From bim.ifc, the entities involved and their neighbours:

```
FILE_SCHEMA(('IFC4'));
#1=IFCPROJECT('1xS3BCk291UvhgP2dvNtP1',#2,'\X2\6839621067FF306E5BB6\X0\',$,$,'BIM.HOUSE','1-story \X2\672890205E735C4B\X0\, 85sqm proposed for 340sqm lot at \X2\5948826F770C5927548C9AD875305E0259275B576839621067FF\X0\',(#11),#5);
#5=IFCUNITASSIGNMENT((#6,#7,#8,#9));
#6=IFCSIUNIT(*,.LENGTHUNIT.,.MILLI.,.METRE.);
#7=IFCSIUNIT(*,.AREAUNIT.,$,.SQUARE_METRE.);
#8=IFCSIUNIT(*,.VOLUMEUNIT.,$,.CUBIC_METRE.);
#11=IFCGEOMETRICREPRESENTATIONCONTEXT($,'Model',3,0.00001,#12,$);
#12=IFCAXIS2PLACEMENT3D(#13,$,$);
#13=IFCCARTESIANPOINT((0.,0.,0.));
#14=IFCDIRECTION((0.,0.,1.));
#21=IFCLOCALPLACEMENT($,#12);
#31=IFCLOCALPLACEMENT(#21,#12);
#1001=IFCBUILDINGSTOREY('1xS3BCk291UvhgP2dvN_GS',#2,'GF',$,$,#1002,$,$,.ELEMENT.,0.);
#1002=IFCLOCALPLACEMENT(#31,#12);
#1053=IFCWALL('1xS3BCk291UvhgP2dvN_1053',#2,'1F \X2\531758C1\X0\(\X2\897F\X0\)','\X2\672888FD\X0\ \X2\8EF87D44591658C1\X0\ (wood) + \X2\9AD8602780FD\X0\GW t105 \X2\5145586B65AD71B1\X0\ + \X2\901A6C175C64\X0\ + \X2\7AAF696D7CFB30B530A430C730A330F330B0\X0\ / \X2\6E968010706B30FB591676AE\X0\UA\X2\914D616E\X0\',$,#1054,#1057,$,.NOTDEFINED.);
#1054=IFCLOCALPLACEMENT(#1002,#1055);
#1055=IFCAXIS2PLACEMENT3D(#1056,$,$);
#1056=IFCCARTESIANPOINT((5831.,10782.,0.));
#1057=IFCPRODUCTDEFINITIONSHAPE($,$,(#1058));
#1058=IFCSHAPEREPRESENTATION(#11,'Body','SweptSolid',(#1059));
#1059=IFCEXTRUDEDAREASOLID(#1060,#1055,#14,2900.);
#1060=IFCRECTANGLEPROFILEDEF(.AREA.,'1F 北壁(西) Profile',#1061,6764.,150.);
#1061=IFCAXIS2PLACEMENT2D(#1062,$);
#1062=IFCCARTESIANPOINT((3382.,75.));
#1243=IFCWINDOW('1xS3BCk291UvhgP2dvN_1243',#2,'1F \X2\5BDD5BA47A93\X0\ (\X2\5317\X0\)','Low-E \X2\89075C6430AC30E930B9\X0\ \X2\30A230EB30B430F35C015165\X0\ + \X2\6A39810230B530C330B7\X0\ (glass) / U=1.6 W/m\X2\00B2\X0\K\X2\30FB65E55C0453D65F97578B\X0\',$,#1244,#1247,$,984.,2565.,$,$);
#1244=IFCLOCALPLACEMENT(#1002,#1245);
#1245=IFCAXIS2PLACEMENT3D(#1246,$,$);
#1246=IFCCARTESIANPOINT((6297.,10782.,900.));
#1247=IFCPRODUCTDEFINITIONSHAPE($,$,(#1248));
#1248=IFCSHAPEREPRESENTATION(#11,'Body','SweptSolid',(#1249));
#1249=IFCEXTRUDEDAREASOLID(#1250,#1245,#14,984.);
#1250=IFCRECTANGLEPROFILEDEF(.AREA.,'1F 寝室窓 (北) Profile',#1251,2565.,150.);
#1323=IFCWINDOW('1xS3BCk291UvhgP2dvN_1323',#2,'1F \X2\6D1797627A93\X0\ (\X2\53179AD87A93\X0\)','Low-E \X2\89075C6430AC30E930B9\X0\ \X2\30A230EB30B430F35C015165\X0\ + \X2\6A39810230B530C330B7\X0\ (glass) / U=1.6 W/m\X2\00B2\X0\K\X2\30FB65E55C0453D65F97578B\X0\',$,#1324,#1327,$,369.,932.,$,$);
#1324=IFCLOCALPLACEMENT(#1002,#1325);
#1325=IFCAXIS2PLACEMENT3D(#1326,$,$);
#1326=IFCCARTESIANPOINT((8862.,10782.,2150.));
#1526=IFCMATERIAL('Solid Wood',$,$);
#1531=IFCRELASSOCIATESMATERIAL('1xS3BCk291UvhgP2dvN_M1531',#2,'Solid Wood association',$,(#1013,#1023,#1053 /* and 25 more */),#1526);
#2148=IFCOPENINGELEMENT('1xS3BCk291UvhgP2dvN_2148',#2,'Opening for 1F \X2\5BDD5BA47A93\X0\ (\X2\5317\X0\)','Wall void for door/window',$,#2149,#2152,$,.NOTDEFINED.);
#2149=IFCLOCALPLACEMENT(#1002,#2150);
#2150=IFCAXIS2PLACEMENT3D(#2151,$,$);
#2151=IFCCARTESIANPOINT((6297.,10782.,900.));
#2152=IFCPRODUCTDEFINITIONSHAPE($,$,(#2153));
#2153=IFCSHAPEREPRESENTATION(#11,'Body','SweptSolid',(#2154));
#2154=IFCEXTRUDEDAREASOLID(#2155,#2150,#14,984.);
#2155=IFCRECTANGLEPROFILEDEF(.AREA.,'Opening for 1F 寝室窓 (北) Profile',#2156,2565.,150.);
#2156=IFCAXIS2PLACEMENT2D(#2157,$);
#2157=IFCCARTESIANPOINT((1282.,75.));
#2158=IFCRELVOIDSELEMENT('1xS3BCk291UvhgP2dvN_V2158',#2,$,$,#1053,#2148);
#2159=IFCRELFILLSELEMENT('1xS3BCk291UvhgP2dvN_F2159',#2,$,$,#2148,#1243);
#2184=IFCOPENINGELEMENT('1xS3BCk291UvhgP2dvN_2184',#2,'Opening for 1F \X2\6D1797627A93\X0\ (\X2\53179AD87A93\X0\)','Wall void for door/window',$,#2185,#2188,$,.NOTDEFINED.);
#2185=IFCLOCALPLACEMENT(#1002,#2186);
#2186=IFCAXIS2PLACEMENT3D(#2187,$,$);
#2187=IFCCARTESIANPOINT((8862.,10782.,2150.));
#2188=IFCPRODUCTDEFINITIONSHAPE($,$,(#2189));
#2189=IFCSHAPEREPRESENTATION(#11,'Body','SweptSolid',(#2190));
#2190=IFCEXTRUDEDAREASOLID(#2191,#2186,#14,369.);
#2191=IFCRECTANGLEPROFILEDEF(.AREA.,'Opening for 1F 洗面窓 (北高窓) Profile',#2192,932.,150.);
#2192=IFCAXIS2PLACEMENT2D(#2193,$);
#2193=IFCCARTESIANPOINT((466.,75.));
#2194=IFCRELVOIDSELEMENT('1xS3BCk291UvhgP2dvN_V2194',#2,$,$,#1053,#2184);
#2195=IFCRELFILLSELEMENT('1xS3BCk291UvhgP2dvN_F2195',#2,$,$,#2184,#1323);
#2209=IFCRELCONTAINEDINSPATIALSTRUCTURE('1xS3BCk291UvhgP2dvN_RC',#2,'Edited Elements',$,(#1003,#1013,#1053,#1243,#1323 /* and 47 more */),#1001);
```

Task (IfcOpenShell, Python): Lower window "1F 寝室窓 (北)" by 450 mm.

```python
import numpy as np
import ifcopenshell
import ifcopenshell.api.geometry
import ifcopenshell.util.placement
import ifcopenshell.util.unit

model = ifcopenshell.open("bim.ifc")
unit_scale = ifcopenshell.util.unit.calculate_unit_scale(model)

window = model.by_guid("1xS3BCk291UvhgP2dvN_1243")
opening = window.FillsVoids[0].RelatingOpeningElement
dz = -0.45 / unit_scale

shift = np.array([0.0, 0.0, dz])
# The window is not placed relative to its opening, so move both.
for product in (opening, window):
    matrix = ifcopenshell.util.placement.get_local_placement(product.ObjectPlacement)
    matrix[:3, 3] += shift
    ifcopenshell.api.geometry.edit_object_placement(model, product=product, matrix=matrix, is_si=False)

print(f"moved by {dz * unit_scale:+.3f} m")

model.write("bim_updated.ifc")
```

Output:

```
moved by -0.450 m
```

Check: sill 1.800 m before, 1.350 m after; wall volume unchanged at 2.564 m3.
